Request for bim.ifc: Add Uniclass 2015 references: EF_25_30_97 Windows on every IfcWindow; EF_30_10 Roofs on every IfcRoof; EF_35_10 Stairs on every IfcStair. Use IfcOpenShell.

First a look at what the model holds.

```python
import ifcopenshell

model = ifcopenshell.open("bim.ifc")
print(model.schema)
print("classifications:", [c.Name for c in model.by_type("IfcClassification")])
for ifc_class in ("IfcDoor", "IfcRoof", "IfcStair", "IfcWall", "IfcWindow"):
    print(ifc_class, len(model.by_type(ifc_class)))
```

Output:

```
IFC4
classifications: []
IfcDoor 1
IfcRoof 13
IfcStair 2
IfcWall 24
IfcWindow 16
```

```python
import ifcopenshell
import ifcopenshell.api.classification

model = ifcopenshell.open("bim.ifc")

system = ifcopenshell.api.classification.add_classification(model, classification="Uniclass 2015")

codes = {
    "IfcWindow": ("EF_25_30_97", "Windows"),
    "IfcRoof": ("EF_30_10", "Roofs"),
    "IfcStair": ("EF_35_10", "Stairs"),
}
for ifc_class, (code, name) in codes.items():
    products = model.by_type(ifc_class)
    ifcopenshell.api.classification.add_reference(
        model, products=products, classification=system, identification=code, name=name
    )
    print(code, len(products))

model.write("bim_v2.ifc")
```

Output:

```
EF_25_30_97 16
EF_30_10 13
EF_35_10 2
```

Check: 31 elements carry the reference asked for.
